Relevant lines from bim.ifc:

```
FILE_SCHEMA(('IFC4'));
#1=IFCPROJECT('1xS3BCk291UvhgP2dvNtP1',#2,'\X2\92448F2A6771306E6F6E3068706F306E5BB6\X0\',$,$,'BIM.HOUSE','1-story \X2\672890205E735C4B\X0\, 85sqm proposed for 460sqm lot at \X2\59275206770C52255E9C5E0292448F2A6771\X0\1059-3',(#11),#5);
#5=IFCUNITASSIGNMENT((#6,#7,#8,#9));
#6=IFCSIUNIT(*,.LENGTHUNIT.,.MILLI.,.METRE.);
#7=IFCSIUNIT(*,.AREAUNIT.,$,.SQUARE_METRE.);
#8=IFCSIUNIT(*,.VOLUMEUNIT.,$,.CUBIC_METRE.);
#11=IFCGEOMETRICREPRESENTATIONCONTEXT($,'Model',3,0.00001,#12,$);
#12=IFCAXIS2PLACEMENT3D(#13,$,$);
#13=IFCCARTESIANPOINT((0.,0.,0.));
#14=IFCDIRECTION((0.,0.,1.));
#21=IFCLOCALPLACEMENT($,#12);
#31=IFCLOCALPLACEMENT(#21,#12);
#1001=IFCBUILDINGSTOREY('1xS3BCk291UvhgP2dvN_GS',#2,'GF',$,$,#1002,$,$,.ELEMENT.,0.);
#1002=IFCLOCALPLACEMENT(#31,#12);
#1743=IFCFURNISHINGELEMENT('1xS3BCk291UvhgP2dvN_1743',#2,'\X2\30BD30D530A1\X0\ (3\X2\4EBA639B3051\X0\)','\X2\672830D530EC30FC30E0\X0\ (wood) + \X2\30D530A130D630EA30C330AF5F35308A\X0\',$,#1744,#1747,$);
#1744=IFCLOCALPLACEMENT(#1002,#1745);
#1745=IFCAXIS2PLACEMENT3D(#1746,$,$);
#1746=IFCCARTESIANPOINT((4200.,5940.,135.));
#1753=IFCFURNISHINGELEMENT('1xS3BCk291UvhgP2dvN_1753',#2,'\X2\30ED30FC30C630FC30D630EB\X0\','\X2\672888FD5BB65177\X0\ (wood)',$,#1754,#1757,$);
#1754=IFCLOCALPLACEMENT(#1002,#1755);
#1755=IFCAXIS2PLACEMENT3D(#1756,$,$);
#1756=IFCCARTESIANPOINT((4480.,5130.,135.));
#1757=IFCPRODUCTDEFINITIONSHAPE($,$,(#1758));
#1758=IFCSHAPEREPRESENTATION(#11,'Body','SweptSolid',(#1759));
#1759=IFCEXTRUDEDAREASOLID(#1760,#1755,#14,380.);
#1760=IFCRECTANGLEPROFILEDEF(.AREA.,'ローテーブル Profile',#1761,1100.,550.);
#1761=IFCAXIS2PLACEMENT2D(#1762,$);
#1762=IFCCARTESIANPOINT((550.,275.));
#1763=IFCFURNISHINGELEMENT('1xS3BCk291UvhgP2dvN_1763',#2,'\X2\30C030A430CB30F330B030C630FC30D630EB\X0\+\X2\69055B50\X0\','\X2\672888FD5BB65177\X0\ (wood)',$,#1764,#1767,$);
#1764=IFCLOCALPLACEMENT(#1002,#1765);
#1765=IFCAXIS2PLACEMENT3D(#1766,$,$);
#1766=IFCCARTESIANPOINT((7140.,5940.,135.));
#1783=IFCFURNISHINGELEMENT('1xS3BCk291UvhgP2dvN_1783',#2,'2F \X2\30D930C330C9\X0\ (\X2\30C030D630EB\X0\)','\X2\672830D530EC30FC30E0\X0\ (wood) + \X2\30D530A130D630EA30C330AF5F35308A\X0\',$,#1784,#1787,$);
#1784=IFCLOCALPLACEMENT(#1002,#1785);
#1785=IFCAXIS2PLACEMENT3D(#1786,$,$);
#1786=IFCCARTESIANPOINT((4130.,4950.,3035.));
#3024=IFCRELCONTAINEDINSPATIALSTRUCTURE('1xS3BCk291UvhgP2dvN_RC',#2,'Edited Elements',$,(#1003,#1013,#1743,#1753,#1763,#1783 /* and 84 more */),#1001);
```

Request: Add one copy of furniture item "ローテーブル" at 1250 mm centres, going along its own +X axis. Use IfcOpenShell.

```python
import ifcopenshell
import ifcopenshell.api.geometry
import ifcopenshell.api.root
import ifcopenshell.util.element
import ifcopenshell.util.placement
import ifcopenshell.util.unit

model = ifcopenshell.open("bim.ifc")
unit_scale = ifcopenshell.util.unit.calculate_unit_scale(model)


def reuse_history(source, copy):
    """copy_class also copies each property set's owner history, people and application; keep the originals."""
    for rel in copy.IsDefinedBy:
        if rel.is_a("IfcRelDefinesByProperties") and (history := rel.RelatingPropertyDefinition.OwnerHistory):
            rel.RelatingPropertyDefinition.OwnerHistory = source.OwnerHistory
            ifcopenshell.util.element.remove_deep2(model, history)


source = model.by_id(1753)
base = ifcopenshell.util.placement.get_local_placement(source.ObjectPlacement)
step = base[:3, 0] * 1.25 / unit_scale

for i in range(1, 2):
    copy = ifcopenshell.api.root.copy_class(model, product=source)
    copy.Representation = ifcopenshell.util.element.copy_deep(
        model, source.Representation, exclude=["IfcGeometricRepresentationContext", "IfcRepresentationMap"]
    )
    reuse_history(source, copy)
    matrix = base.copy()
    matrix[:3, 3] += i * step
    print("added at", matrix[:3, 3].round(3) + 0.0)
    ifcopenshell.api.geometry.edit_object_placement(model, product=copy, matrix=matrix, is_si=False)

model.write("bim_updated.ifc")
```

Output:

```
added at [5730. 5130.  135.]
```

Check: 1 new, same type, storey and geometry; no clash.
